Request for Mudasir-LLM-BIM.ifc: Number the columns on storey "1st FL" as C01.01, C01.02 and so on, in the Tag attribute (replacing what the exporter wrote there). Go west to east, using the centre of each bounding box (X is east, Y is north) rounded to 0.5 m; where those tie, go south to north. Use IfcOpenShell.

First a look at what the model holds.

```python
import ifcopenshell
import ifcopenshell.util.element
import ifcopenshell.util.placement

model = ifcopenshell.open("Mudasir-LLM-BIM.ifc")
print(model.schema)
storey = next(s for s in model.by_type("IfcBuildingStorey") if s.Name == "1st FL")
columns = [e for e in ifcopenshell.util.element.get_decomposition(storey) if e.is_a("IfcColumn")]
for e in sorted(columns, key=lambda e: e.id()):
    origin = ifcopenshell.util.placement.get_local_placement(e.ObjectPlacement)[:3, 3]
    print(e.id(), e.Tag, e.Name, origin.round(2) + 0.0, sep=" | ")
```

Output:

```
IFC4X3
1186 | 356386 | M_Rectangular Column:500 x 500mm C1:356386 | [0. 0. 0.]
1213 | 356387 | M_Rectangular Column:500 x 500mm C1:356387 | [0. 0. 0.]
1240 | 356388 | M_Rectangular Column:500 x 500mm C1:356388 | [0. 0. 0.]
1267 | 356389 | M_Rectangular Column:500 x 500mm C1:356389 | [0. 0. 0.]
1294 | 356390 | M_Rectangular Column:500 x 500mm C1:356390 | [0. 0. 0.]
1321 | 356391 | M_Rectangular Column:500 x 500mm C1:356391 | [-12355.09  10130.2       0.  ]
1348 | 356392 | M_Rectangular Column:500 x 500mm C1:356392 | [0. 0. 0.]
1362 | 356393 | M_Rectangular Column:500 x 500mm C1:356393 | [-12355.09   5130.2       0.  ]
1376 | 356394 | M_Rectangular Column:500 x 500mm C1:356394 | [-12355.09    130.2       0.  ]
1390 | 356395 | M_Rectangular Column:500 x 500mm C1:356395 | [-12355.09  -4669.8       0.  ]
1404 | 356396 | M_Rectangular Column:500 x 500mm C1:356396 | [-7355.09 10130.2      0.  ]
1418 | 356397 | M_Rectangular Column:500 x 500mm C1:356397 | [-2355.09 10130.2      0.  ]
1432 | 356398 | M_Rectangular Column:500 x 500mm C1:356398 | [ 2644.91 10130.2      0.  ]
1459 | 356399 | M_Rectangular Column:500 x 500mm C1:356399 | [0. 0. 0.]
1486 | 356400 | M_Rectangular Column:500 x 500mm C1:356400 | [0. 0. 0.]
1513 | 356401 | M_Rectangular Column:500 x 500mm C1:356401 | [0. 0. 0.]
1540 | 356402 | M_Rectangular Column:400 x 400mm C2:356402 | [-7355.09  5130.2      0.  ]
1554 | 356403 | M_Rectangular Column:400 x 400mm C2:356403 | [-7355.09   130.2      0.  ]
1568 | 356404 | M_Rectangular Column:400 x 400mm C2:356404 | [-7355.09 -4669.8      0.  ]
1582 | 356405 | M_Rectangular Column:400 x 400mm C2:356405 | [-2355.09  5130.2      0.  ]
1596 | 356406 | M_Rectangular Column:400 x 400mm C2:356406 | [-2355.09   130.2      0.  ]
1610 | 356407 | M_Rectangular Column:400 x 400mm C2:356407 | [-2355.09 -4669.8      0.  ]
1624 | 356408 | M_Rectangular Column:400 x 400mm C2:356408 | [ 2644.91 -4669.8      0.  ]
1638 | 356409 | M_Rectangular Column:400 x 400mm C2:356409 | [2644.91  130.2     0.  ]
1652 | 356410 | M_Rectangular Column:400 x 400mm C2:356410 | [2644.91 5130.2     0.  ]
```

```python
import ifcopenshell
import ifcopenshell.geom
import ifcopenshell.util.element
import ifcopenshell.util.shape

model = ifcopenshell.open("Mudasir-LLM-BIM.ifc")
settings = ifcopenshell.geom.settings()
settings.set("use-world-coords", True)


def centre(element):
    shape = ifcopenshell.geom.create_shape(settings, element)
    return ifcopenshell.util.shape.get_bbox_centroid(shape.geometry)


storey = next(s for s in model.by_type("IfcBuildingStorey") if s.Name == "1st FL")
columns = [e for e in ifcopenshell.util.element.get_decomposition(storey) if e.is_a("IfcColumn")]

# Insertion points can sit at a corner or the storey origin, so sort by the geometry (in metres).
centres = {e: centre(e) for e in columns}
columns.sort(key=lambda e: (round(centres[e][0] / 0.5), centres[e][1]))

for i, e in enumerate(columns, start=1):
    number = f"C01.{i:02d}"
    e.Tag = number
    print(e.id(), number)

model.write("Mudasir-LLM-BIM_rev.ifc")
```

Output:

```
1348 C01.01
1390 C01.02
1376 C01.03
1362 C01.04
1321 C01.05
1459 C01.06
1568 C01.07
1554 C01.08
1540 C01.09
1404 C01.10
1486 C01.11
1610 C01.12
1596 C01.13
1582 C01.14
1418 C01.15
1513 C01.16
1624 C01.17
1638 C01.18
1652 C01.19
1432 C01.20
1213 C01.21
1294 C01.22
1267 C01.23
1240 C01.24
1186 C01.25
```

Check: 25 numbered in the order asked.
